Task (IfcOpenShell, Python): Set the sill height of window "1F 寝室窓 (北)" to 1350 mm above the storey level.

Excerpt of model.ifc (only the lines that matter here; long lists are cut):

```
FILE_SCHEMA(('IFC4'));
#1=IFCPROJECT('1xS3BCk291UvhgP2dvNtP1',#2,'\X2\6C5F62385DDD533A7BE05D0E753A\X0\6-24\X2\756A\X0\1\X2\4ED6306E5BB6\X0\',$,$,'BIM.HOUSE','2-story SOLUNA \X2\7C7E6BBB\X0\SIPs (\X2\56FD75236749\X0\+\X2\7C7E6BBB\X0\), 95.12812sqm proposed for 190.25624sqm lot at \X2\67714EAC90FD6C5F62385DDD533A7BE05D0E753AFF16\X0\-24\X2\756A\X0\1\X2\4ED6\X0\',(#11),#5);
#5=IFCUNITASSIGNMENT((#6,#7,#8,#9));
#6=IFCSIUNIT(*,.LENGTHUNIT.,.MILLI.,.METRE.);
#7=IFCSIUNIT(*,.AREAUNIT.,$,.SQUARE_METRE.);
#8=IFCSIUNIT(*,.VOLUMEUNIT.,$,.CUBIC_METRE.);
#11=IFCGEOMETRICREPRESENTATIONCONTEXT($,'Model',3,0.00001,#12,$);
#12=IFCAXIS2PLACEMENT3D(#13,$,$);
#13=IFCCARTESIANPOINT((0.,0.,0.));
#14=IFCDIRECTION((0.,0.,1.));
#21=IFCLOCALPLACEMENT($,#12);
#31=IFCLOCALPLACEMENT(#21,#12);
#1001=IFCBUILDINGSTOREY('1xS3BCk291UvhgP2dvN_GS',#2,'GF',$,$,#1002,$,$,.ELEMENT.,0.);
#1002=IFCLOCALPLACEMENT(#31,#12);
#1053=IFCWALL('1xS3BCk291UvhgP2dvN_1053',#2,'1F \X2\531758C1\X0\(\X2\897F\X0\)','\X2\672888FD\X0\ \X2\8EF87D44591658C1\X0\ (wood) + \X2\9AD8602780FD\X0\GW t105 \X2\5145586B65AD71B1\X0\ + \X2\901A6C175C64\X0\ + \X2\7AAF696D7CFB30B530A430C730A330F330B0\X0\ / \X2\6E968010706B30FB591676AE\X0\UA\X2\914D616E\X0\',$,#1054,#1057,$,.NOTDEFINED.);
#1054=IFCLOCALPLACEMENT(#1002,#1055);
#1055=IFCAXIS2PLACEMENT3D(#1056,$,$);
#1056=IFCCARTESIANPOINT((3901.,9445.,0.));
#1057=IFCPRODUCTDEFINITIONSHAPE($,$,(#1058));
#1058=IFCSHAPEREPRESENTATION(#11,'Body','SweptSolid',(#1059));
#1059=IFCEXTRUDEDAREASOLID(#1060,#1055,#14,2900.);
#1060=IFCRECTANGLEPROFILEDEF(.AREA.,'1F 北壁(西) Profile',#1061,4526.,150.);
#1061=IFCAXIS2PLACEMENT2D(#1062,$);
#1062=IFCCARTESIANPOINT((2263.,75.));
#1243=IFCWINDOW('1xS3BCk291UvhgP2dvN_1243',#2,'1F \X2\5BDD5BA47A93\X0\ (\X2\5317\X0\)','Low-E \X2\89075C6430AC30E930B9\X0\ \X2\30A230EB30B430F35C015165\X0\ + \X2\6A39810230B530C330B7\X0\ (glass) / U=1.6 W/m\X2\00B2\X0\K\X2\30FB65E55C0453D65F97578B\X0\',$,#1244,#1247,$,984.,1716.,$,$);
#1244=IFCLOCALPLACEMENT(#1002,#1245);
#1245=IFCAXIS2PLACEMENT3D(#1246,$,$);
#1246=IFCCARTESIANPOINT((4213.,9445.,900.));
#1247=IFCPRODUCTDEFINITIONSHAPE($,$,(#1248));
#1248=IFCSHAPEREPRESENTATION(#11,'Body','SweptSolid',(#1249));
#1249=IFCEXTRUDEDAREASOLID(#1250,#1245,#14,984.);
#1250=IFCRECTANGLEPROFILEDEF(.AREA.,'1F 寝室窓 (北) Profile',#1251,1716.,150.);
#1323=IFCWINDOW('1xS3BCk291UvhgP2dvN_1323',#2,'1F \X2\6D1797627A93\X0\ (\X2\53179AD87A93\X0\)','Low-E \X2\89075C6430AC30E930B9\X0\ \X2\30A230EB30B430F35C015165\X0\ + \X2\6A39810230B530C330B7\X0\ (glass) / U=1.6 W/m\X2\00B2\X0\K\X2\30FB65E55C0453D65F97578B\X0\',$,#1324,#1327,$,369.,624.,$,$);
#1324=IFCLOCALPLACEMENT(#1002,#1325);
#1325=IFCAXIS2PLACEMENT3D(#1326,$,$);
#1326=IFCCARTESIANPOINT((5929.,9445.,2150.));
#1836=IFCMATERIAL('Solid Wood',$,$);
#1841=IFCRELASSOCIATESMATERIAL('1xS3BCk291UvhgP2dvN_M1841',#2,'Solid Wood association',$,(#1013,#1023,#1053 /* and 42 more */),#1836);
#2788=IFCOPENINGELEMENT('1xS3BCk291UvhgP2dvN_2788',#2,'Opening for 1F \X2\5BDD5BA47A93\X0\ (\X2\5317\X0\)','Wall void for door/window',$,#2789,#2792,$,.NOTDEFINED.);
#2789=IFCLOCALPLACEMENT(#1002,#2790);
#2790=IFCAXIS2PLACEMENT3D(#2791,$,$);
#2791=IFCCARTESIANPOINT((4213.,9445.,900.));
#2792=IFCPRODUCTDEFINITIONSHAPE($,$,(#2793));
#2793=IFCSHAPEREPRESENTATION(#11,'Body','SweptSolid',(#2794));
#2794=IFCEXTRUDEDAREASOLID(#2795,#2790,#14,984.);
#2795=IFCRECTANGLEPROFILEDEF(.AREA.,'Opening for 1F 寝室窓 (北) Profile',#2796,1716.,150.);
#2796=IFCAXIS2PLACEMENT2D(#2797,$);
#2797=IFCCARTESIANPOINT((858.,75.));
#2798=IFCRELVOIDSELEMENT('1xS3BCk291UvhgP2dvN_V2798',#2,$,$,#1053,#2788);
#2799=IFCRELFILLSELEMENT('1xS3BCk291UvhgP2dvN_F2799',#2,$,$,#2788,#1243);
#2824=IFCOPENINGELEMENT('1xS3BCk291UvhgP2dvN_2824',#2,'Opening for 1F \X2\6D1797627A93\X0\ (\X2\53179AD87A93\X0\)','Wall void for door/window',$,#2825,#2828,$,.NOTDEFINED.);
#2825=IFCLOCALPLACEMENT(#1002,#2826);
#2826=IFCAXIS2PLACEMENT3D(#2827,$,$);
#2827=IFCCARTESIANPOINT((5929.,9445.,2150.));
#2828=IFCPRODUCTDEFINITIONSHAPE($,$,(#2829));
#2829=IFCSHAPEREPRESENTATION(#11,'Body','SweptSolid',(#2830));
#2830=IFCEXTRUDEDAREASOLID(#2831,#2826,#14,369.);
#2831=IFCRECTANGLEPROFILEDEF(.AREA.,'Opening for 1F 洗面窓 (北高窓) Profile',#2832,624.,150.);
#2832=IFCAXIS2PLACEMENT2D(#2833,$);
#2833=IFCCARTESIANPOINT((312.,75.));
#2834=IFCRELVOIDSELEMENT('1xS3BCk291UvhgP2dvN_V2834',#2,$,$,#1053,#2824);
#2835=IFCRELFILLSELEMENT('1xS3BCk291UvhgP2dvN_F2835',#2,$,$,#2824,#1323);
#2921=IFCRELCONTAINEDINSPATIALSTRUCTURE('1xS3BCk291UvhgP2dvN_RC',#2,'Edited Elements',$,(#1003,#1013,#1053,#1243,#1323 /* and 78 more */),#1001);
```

```python
import numpy as np
import ifcopenshell
import ifcopenshell.api.geometry
import ifcopenshell.geom
import ifcopenshell.util.element
import ifcopenshell.util.placement
import ifcopenshell.util.shape
import ifcopenshell.util.unit

model = ifcopenshell.open("model.ifc")
unit_scale = ifcopenshell.util.unit.calculate_unit_scale(model)

window = model.by_guid("1xS3BCk291UvhgP2dvN_1243")
opening = window.FillsVoids[0].RelatingOpeningElement
storey = ifcopenshell.util.element.get_container(window, ifc_class="IfcBuildingStorey")
level = ifcopenshell.util.placement.get_local_placement(storey.ObjectPlacement)[2, 3]

# The opening's origin need not be at the sill, so measure its lowest point.
shape = ifcopenshell.geom.create_shape(ifcopenshell.geom.settings(), opening)
bottom = ifcopenshell.util.shape.get_shape_bottom_elevation(shape, shape.geometry) / unit_scale
dz = level + 1350.0 - bottom

shift = np.array([0.0, 0.0, dz])
# The window is not placed relative to its opening, so move both.
for product in (opening, window):
    matrix = ifcopenshell.util.placement.get_local_placement(product.ObjectPlacement)
    matrix[:3, 3] += shift
    ifcopenshell.api.geometry.edit_object_placement(model, product=product, matrix=matrix, is_si=False)

print(f"moved by {dz * unit_scale:+.3f} m")

model.write("model_edited.ifc")
```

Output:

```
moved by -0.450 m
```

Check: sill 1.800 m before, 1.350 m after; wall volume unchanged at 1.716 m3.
